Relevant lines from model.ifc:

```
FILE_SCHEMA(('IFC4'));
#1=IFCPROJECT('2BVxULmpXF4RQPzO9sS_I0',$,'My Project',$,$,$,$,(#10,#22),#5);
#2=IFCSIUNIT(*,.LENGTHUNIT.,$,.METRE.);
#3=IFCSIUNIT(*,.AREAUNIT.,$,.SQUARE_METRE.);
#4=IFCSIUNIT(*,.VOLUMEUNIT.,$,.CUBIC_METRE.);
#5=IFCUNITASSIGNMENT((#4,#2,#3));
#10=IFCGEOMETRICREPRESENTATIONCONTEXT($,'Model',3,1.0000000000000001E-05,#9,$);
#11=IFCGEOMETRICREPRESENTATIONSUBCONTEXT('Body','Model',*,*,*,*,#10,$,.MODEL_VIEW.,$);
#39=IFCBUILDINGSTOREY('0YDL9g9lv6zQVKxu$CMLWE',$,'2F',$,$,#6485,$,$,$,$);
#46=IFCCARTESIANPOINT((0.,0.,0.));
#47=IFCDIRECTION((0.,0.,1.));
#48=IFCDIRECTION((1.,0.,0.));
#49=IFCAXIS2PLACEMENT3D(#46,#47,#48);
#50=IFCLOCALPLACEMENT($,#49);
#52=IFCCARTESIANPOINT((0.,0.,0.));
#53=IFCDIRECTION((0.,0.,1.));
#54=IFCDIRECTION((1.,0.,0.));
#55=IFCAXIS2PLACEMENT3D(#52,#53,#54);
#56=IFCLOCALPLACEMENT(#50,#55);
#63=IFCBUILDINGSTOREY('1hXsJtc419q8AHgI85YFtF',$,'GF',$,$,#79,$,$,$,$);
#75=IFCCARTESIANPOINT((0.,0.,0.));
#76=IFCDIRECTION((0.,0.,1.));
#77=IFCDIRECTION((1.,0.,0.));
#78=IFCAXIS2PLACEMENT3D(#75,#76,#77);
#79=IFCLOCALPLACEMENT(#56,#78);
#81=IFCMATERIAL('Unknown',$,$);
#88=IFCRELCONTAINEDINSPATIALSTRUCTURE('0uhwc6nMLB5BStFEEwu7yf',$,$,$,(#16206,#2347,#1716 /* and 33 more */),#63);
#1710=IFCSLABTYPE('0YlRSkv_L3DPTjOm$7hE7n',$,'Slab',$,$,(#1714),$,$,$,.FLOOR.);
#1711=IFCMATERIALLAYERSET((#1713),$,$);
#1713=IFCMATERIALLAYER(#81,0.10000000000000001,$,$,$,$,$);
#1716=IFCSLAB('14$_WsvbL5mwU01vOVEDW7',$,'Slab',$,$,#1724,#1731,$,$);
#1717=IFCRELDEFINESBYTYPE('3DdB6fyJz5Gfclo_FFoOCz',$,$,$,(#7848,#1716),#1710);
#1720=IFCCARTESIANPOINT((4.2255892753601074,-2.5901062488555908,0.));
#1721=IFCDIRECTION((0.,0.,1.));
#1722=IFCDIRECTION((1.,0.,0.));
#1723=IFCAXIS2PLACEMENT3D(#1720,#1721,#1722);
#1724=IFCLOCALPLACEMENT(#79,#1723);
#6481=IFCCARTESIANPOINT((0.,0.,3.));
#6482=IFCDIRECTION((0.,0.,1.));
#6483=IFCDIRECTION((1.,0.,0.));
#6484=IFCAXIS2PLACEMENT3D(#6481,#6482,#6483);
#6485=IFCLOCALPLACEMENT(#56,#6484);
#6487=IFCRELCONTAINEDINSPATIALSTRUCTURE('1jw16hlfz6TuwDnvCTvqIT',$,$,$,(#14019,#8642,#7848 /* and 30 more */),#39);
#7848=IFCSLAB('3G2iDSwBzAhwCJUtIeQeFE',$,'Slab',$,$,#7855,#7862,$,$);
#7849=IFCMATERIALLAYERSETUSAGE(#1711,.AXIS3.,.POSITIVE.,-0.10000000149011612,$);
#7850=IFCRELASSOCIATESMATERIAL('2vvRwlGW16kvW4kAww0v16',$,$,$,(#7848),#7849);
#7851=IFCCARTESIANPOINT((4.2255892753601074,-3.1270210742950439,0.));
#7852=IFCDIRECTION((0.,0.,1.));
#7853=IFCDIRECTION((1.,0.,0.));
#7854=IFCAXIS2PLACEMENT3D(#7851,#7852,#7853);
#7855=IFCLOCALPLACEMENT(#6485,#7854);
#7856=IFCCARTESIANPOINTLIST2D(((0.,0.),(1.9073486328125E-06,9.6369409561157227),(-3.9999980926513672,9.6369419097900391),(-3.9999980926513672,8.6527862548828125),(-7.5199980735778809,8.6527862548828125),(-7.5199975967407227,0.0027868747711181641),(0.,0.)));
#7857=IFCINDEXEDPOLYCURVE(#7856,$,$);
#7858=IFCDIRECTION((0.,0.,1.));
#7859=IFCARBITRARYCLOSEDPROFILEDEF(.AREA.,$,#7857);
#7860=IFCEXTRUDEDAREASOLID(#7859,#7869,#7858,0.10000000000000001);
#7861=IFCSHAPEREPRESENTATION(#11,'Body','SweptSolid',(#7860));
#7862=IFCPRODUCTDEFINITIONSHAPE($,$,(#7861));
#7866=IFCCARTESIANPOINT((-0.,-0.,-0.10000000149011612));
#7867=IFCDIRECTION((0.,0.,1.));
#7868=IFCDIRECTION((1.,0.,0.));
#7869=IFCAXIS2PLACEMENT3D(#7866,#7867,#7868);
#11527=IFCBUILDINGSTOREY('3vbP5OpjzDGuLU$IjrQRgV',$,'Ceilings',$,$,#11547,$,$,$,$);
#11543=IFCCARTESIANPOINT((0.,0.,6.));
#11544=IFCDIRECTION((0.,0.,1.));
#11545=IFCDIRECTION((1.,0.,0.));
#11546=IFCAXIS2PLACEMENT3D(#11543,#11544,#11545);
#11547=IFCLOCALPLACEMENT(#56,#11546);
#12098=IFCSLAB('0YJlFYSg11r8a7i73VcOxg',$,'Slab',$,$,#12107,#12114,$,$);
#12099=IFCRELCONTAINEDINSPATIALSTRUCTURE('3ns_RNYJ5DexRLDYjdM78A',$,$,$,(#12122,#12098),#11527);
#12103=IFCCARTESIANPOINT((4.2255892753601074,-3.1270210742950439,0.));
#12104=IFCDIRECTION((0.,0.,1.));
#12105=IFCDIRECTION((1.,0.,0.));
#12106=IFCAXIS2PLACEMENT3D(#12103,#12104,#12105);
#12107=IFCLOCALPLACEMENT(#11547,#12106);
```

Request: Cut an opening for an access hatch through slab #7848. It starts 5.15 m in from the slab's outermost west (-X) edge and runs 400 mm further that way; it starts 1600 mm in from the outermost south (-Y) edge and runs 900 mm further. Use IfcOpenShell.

```python
import numpy as np
import ifcopenshell
import ifcopenshell.api.feature
import ifcopenshell.api.geometry
import ifcopenshell.api.root
import ifcopenshell.geom
import ifcopenshell.util.placement
import ifcopenshell.util.representation
import ifcopenshell.util.shape
import ifcopenshell.util.unit

model = ifcopenshell.open("model.ifc")
unit_scale = ifcopenshell.util.unit.calculate_unit_scale(model)
settings = ifcopenshell.geom.settings()


def volume(element):
    """Net volume in cubic metres, openings subtracted."""
    shape = ifcopenshell.geom.create_shape(settings, element)
    return ifcopenshell.util.shape.get_volume(shape.geometry)


slab = model.by_id(7848)
before = volume(slab)

# Extent in the slab's own axes, in metres. The edges named are its -X and -Y sides.
slab_shape = ifcopenshell.geom.create_shape(settings, slab)
vertices = ifcopenshell.util.shape.get_vertices(slab_shape.geometry)
x_min, y_min, bottom = vertices.min(axis=0)
top = vertices[:, 2].max()

opening = ifcopenshell.api.root.create_entity(model, ifc_class="IfcOpeningElement", name="Access hatch opening", predefined_type="OPENING")
context = ifcopenshell.util.representation.get_context(model, "Model", "Body", "MODEL_VIEW")
width, depth = 0.4, 0.9
outline = [(0.0, 0.0), (width, 0.0), (width, depth), (0.0, depth), (0.0, 0.0)]
# Overshoot both faces by 50 mm so the cut is clean.
shape = ifcopenshell.api.geometry.add_slab_representation(
    model, context=context, depth=top - bottom + 0.1, polyline=outline
)
ifcopenshell.api.geometry.assign_representation(model, product=opening, representation=shape)

matrix = ifcopenshell.util.placement.get_local_placement(slab.ObjectPlacement)
matrix[:, 3] = matrix @ np.append(np.array([x_min + 5.15, y_min + 1.6, bottom - 0.05]) / unit_scale, 1.0)
ifcopenshell.api.geometry.edit_object_placement(model, product=opening, matrix=matrix, is_si=False)
ifcopenshell.api.feature.add_feature(model, feature=opening, element=slab)

after = volume(slab)

print(f"slab volume {before:.3f} -> {after:.3f} m3")

model.write("model_updated.ifc")
```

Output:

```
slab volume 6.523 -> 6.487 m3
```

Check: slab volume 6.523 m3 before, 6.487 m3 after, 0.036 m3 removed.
